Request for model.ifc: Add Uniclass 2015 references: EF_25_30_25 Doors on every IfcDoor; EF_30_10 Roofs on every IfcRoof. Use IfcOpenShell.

First a look at what the model holds.

```python
import ifcopenshell

model = ifcopenshell.open("model.ifc")
print(model.schema)
print("classifications:", [c.Name for c in model.by_type("IfcClassification")])
for ifc_class in ("IfcDoor", "IfcRoof", "IfcStair", "IfcWall", "IfcWindow"):
    print(ifc_class, len(model.by_type(ifc_class)))
```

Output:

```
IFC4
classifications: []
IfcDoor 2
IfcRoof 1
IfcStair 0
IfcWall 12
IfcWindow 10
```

```python
import ifcopenshell
import ifcopenshell.api.classification

model = ifcopenshell.open("model.ifc")

system = ifcopenshell.api.classification.add_classification(model, classification="Uniclass 2015")

codes = {
    "IfcDoor": ("EF_25_30_25", "Doors"),
    "IfcRoof": ("EF_30_10", "Roofs"),
}
for ifc_class, (code, name) in codes.items():
    products = model.by_type(ifc_class)
    ifcopenshell.api.classification.add_reference(
        model, products=products, classification=system, identification=code, name=name
    )
    print(code, len(products))

model.write("model-out.ifc")
```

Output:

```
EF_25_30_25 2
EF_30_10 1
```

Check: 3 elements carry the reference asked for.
